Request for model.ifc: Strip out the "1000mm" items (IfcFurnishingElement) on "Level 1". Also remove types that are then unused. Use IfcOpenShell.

First a look at what the model holds.

```python
import ifcopenshell
import ifcopenshell.util.element

model = ifcopenshell.open("model.ifc")
print(model.schema)
storey = next(s for s in model.by_type("IfcBuildingStorey") if s.Name == "Level 1")
furniture = [e for e in ifcopenshell.util.element.get_decomposition(storey) if e.is_a("IfcFurnishingElement")]
seen = {}
for e in furniture:
    element_type = ifcopenshell.util.element.get_type(e)
    name = element_type.Name if element_type not in (None, e) else None
    seen[name] = seen.get(name, 0) + 1
for name, count in sorted(seen.items(), key=str):
    print(count, "x", name)
```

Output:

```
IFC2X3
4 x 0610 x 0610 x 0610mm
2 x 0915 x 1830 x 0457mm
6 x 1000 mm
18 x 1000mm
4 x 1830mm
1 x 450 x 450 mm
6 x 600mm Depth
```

```python
import ifcopenshell
import ifcopenshell.api.root
import ifcopenshell.util.element

model = ifcopenshell.open("model.ifc")

storey = next(s for s in model.by_type("IfcBuildingStorey") if s.Name == "Level 1")
furniture = [e for e in ifcopenshell.util.element.get_decomposition(storey) if e.is_a("IfcFurnishingElement")]
targets = [e for e in furniture if (t := ifcopenshell.util.element.get_type(e)) not in (None, e) and t.Name == "1000mm"]
types = {ifcopenshell.util.element.get_type(e) for e in targets} - {None, *targets}

for e in targets:
    ifcopenshell.api.root.remove_product(model, product=e)
print(len(targets), "removed")

unused = [t for t in types if not ifcopenshell.util.element.get_types(t)]
for t in unused:
    ifcopenshell.api.root.remove_product(model, product=t)
print(len(unused), "unused types removed")

model.write("model_rev.ifc")
```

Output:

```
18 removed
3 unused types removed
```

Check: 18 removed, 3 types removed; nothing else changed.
